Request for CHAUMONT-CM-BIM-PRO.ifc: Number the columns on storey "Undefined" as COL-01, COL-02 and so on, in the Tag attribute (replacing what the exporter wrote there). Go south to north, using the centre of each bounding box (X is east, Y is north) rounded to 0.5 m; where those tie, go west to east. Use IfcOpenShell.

First a look at what the model holds.

```python
import ifcopenshell
import ifcopenshell.util.element
import ifcopenshell.util.placement

model = ifcopenshell.open("CHAUMONT-CM-BIM-PRO.ifc")
print(model.schema)
storey = next(s for s in model.by_type("IfcBuildingStorey") if s.Name == "Undefined")
columns = [e for e in ifcopenshell.util.element.get_decomposition(storey) if e.is_a("IfcColumn")]
for e in sorted(columns, key=lambda e: e.id()):
    origin = ifcopenshell.util.placement.get_local_placement(e.ObjectPlacement)[:3, 3]
    print(e.id(), e.Tag, e.Name, origin.round(2) + 0.0, sep=" | ")
```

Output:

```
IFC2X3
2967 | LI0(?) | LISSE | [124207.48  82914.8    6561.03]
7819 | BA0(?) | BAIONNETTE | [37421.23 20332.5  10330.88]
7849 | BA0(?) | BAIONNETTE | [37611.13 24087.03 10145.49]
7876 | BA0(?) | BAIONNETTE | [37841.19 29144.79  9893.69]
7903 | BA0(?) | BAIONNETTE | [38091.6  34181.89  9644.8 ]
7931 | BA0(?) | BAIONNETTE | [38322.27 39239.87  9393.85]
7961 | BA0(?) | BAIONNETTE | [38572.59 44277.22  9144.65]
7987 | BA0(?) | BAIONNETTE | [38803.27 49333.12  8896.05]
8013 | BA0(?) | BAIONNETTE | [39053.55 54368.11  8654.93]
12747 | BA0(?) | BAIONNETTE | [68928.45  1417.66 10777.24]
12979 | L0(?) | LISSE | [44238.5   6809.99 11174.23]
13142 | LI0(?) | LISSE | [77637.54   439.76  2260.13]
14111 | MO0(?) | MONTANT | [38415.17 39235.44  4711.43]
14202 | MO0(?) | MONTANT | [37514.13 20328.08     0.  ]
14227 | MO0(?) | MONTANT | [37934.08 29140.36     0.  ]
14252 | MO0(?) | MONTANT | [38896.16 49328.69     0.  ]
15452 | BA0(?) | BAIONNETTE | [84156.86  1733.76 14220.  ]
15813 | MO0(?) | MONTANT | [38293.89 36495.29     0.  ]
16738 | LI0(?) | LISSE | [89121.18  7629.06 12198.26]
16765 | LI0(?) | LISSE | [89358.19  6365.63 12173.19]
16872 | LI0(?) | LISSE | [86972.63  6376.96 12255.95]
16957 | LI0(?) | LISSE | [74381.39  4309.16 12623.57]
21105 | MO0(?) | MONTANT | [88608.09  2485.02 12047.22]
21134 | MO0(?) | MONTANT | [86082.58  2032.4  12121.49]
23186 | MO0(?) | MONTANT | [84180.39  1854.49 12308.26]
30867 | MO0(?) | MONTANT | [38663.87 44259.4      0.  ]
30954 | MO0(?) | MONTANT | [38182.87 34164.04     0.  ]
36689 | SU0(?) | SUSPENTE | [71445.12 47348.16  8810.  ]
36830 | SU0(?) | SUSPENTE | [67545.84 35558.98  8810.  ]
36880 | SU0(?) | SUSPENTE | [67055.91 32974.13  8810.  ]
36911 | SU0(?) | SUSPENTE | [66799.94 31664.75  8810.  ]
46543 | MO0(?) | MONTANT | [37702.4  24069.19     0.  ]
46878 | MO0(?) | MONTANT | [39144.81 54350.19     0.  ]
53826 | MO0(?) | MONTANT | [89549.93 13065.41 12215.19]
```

```python
import ifcopenshell
import ifcopenshell.geom
import ifcopenshell.util.element
import ifcopenshell.util.shape

model = ifcopenshell.open("CHAUMONT-CM-BIM-PRO.ifc")
settings = ifcopenshell.geom.settings()
settings.set("use-world-coords", True)


def centre(element):
    shape = ifcopenshell.geom.create_shape(settings, element)
    return ifcopenshell.util.shape.get_bbox_centroid(shape.geometry)


storey = next(s for s in model.by_type("IfcBuildingStorey") if s.Name == "Undefined")
columns = [e for e in ifcopenshell.util.element.get_decomposition(storey) if e.is_a("IfcColumn")]

# Insertion points can sit at a corner or the storey origin, so sort by the geometry (in metres).
centres = {e: centre(e) for e in columns}
columns.sort(key=lambda e: (round(centres[e][1] / 0.5), centres[e][0]))

for i, e in enumerate(columns, start=1):
    number = f"COL-{i:02d}"
    e.Tag = number
    print(e.id(), number)

model.write("CHAUMONT-CM-BIM-PRO-out.ifc")
```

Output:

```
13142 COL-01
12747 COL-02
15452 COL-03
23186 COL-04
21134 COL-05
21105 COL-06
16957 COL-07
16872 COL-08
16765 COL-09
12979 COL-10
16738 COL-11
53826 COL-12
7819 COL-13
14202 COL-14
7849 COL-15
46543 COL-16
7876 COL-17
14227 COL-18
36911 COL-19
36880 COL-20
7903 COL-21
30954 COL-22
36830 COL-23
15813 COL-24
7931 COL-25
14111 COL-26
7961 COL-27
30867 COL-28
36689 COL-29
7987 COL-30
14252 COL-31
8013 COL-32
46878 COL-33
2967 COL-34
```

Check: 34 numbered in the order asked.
